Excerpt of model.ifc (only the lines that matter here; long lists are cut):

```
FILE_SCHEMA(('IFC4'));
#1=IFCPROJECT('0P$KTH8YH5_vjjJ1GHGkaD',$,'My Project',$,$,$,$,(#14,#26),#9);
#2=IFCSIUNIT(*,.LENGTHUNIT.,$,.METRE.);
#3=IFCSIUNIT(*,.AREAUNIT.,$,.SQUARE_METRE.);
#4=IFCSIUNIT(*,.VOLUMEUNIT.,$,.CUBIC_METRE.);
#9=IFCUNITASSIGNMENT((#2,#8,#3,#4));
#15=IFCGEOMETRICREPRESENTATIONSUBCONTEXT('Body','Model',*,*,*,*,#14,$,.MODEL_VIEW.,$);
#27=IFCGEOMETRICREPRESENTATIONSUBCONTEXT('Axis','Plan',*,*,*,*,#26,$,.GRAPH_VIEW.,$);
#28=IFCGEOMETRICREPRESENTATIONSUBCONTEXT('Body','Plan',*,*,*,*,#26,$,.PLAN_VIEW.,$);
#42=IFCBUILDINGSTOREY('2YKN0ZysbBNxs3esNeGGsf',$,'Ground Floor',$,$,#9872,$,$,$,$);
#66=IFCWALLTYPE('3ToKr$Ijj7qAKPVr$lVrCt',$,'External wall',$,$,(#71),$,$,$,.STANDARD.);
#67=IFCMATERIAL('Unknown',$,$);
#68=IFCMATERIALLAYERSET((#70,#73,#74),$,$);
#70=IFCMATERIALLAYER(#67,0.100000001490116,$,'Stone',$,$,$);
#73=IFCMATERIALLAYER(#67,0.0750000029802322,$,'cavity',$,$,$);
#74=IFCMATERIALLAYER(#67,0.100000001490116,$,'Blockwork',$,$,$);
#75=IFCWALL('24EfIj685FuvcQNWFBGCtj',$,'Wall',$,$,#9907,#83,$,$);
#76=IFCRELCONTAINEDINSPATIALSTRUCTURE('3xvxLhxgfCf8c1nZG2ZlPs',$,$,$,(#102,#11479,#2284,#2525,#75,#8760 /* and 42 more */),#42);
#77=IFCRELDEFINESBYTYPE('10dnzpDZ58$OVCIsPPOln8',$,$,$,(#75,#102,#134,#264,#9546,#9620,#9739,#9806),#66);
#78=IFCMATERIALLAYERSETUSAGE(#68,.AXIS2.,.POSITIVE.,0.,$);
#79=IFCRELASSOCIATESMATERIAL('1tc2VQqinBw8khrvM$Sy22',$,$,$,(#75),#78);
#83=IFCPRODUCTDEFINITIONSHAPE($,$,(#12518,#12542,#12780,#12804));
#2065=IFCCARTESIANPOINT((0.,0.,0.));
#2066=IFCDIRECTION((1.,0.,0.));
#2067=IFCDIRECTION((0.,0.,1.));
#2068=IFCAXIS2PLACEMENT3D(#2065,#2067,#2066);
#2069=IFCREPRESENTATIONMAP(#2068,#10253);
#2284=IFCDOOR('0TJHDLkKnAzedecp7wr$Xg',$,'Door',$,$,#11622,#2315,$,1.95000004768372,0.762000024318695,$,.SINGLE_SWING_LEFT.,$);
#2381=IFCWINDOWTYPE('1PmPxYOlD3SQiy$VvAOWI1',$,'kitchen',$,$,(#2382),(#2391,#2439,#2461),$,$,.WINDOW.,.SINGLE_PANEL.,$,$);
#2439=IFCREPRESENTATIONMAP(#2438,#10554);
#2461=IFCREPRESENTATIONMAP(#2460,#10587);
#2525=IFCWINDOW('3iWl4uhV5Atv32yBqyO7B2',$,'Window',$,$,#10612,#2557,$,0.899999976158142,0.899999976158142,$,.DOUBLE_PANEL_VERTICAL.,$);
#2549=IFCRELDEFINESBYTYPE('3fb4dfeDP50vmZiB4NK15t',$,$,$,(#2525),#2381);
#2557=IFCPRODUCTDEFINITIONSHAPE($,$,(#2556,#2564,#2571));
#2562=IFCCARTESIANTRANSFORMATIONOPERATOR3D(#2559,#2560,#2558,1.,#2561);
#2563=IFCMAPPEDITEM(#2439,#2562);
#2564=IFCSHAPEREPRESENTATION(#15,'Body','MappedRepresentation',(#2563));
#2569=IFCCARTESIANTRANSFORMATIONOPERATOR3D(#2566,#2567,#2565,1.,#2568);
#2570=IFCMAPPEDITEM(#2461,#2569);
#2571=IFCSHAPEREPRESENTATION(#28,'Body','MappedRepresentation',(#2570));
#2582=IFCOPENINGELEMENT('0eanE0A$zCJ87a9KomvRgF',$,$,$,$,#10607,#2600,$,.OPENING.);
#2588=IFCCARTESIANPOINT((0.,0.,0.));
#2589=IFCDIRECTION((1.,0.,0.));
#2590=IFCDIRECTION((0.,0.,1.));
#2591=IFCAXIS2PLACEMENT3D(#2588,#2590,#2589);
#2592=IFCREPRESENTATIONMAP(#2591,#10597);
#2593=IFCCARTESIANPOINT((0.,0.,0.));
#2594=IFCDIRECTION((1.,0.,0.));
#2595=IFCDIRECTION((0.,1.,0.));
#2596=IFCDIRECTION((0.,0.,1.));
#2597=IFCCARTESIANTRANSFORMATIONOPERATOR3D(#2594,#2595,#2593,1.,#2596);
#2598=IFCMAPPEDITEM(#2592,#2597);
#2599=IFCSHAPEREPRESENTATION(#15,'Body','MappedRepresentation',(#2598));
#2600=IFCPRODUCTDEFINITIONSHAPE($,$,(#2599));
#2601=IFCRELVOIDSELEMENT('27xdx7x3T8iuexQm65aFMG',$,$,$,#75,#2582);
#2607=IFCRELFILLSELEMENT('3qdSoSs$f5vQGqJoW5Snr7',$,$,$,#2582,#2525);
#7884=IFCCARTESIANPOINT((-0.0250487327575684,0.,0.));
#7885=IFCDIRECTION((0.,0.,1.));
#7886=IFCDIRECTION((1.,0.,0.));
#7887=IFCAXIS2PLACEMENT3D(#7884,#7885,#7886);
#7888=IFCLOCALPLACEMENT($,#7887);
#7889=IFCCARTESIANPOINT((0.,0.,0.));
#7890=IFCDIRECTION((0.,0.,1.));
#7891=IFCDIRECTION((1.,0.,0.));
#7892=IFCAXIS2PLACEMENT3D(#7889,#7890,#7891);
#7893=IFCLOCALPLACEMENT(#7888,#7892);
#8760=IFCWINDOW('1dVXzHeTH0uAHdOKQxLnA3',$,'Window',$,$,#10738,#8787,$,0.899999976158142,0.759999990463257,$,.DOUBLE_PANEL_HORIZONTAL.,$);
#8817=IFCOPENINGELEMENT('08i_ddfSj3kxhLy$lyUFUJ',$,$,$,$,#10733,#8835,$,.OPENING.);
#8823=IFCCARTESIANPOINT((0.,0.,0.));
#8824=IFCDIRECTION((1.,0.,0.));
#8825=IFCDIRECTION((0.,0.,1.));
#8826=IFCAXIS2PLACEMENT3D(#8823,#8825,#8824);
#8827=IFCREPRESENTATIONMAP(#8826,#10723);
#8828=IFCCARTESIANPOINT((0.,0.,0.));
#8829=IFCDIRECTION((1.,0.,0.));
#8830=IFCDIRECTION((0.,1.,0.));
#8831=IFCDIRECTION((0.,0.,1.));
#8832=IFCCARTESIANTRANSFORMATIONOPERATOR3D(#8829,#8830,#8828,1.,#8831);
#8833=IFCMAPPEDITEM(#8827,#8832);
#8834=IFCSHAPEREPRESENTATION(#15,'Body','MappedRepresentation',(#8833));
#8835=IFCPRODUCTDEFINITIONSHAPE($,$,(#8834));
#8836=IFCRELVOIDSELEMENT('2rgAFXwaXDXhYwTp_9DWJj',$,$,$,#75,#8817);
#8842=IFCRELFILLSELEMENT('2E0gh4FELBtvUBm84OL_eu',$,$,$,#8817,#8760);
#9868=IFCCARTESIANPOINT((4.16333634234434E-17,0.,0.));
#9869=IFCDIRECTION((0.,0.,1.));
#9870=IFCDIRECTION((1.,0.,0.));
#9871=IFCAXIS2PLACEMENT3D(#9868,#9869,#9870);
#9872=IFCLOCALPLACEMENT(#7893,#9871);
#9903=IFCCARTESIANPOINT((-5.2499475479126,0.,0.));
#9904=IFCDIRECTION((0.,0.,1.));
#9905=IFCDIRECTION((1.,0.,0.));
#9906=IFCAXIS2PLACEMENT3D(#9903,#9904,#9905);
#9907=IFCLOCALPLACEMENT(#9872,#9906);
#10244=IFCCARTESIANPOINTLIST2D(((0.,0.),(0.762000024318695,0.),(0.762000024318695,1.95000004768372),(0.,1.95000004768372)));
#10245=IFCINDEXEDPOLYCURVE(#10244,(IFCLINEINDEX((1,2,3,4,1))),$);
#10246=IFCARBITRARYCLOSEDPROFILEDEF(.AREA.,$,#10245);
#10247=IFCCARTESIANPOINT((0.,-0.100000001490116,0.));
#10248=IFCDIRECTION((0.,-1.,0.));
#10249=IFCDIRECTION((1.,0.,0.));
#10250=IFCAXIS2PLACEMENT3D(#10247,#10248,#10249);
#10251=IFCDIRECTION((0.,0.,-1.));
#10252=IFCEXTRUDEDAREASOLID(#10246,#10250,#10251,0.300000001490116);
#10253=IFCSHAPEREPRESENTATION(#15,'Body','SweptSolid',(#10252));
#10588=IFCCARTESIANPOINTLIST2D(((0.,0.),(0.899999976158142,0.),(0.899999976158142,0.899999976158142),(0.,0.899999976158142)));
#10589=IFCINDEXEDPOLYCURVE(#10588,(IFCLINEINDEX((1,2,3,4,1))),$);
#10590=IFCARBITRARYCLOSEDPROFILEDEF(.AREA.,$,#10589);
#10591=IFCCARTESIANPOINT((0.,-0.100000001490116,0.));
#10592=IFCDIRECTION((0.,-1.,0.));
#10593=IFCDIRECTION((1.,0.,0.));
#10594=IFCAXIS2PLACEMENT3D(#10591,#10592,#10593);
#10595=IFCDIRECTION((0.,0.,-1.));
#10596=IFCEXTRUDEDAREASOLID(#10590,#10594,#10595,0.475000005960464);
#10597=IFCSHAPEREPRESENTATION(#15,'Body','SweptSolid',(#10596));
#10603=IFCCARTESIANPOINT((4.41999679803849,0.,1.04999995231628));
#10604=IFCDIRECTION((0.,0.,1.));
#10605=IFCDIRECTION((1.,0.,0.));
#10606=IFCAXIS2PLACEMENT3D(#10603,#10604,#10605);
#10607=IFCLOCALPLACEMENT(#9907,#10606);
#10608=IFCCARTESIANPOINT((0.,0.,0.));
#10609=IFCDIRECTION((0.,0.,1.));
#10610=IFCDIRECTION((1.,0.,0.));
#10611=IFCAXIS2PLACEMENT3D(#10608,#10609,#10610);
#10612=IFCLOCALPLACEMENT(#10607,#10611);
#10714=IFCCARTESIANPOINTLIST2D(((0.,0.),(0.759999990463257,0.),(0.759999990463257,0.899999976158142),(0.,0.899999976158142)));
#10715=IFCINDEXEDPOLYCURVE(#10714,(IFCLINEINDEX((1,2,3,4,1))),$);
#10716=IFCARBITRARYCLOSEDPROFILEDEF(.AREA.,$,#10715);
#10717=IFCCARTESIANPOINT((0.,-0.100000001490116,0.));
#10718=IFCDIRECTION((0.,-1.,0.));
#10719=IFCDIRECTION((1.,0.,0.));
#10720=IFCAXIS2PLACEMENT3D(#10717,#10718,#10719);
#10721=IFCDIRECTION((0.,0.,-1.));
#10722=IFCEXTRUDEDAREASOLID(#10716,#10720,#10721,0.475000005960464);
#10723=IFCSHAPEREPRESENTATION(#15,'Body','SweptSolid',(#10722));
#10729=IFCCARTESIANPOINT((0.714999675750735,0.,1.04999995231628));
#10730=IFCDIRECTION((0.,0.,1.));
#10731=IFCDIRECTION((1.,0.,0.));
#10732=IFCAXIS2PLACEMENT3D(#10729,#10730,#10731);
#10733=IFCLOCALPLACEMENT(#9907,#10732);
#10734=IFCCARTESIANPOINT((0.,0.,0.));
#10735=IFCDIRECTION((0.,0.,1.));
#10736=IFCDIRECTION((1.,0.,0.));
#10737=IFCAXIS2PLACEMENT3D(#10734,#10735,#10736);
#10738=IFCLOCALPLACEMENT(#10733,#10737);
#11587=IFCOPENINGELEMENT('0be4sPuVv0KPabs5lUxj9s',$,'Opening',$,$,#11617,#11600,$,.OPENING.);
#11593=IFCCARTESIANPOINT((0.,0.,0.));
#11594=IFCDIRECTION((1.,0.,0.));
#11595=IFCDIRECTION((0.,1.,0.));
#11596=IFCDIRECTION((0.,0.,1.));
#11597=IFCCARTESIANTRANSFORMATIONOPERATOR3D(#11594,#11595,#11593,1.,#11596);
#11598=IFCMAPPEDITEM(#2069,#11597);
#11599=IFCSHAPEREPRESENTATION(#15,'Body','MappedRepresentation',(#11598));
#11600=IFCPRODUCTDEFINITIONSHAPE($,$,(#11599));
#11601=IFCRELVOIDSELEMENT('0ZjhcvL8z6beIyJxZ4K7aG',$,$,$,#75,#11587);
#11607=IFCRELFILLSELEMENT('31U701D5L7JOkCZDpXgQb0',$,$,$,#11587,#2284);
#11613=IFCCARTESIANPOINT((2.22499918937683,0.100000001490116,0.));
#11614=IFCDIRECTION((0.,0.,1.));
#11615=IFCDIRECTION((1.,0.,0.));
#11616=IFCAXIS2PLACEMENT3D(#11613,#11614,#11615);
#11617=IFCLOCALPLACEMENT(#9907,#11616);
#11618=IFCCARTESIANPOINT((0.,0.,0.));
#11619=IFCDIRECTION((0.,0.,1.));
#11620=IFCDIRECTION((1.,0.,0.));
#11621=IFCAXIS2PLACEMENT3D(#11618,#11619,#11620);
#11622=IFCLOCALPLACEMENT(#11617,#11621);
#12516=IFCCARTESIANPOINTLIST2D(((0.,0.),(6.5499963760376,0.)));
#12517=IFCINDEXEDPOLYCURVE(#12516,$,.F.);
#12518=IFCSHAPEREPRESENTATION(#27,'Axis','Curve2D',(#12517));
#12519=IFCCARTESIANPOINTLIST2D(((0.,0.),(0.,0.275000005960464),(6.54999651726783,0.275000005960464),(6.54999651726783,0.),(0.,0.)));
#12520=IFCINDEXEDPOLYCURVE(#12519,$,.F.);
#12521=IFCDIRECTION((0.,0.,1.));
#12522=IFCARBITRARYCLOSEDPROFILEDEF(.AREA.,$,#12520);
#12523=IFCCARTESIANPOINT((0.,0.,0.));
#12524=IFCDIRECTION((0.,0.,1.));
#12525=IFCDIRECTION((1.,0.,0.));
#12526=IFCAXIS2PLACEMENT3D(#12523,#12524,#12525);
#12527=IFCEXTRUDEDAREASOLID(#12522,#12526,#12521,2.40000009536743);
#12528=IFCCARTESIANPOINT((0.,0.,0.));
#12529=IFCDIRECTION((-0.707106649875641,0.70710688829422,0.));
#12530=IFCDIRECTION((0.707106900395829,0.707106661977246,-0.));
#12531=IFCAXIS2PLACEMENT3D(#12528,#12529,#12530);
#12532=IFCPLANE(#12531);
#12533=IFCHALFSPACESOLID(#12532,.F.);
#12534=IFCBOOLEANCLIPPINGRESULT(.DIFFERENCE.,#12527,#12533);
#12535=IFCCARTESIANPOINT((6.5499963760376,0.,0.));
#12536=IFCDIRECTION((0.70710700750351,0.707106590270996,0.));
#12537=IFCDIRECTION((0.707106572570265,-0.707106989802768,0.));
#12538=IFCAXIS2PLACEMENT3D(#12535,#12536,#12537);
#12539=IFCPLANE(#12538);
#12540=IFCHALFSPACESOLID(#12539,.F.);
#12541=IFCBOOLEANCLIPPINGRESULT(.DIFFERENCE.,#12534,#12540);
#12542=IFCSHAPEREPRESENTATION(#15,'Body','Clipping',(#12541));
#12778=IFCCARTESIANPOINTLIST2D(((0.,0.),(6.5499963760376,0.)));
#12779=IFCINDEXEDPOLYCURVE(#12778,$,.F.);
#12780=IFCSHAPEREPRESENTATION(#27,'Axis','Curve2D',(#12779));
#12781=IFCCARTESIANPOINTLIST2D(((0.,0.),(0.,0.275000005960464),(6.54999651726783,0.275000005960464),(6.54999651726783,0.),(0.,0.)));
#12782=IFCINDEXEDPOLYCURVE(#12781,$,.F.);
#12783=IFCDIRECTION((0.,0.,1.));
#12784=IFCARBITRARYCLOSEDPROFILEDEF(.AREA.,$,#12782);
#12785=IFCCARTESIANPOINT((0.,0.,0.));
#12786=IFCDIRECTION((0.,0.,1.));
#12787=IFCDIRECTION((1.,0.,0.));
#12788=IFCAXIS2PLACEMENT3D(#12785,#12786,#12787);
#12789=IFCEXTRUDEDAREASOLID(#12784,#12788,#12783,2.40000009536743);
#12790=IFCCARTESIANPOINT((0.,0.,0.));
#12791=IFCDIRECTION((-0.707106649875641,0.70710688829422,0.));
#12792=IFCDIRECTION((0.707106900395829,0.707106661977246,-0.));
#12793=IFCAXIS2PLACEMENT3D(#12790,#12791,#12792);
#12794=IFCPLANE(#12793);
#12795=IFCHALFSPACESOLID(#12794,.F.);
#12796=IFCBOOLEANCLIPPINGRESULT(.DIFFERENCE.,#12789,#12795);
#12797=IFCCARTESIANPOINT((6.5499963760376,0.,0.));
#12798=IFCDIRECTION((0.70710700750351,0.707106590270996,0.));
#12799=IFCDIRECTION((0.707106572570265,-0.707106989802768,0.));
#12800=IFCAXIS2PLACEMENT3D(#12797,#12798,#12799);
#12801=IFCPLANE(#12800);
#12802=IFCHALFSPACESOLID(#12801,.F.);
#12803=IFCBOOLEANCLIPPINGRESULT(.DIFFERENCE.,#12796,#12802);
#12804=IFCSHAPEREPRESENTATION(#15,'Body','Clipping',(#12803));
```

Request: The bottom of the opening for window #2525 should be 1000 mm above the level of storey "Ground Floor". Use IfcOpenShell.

```python
import numpy as np
import ifcopenshell
import ifcopenshell.api.geometry
import ifcopenshell.geom
import ifcopenshell.util.element
import ifcopenshell.util.placement
import ifcopenshell.util.shape
import ifcopenshell.util.unit

model = ifcopenshell.open("model.ifc")
unit_scale = ifcopenshell.util.unit.calculate_unit_scale(model)

window = model.by_guid("3iWl4uhV5Atv32yBqyO7B2")
opening = window.FillsVoids[0].RelatingOpeningElement
storey = ifcopenshell.util.element.get_container(window, ifc_class="IfcBuildingStorey")
level = ifcopenshell.util.placement.get_local_placement(storey.ObjectPlacement)[2, 3]

# The opening's origin need not be at the sill, so measure its lowest point.
shape = ifcopenshell.geom.create_shape(ifcopenshell.geom.settings(), opening)
bottom = ifcopenshell.util.shape.get_shape_bottom_elevation(shape, shape.geometry) / unit_scale
dz = level + 1.0 - bottom

shift = np.array([0.0, 0.0, dz])
# The window is placed relative to its opening, so it follows when the opening moves.
matrix = ifcopenshell.util.placement.get_local_placement(opening.ObjectPlacement)
matrix[:3, 3] += shift
ifcopenshell.api.geometry.edit_object_placement(
    model, product=opening, matrix=matrix, is_si=False, should_transform_children=True
)

print(f"moved by {dz * unit_scale:+.3f} m")

model.write("model_updated.ifc")
```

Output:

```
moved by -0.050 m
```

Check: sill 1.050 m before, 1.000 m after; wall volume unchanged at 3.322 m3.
